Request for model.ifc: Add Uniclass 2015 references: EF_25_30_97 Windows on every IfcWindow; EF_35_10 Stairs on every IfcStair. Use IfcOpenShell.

First a look at what the model holds.

```python
import ifcopenshell

model = ifcopenshell.open("model.ifc")
print(model.schema)
print("classifications:", [c.Name for c in model.by_type("IfcClassification")])
for ifc_class in ("IfcDoor", "IfcRoof", "IfcStair", "IfcWall", "IfcWindow"):
    print(ifc_class, len(model.by_type(ifc_class)))
```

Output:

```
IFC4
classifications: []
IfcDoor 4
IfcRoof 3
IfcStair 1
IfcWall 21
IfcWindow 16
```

```python
import ifcopenshell
import ifcopenshell.api.classification

model = ifcopenshell.open("model.ifc")

system = ifcopenshell.api.classification.add_classification(model, classification="Uniclass 2015")

codes = {
    "IfcWindow": ("EF_25_30_97", "Windows"),
    "IfcStair": ("EF_35_10", "Stairs"),
}
for ifc_class, (code, name) in codes.items():
    products = model.by_type(ifc_class)
    ifcopenshell.api.classification.add_reference(
        model, products=products, classification=system, identification=code, name=name
    )
    print(code, len(products))

model.write("model_updated.ifc")
```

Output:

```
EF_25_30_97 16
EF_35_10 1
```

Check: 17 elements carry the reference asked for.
